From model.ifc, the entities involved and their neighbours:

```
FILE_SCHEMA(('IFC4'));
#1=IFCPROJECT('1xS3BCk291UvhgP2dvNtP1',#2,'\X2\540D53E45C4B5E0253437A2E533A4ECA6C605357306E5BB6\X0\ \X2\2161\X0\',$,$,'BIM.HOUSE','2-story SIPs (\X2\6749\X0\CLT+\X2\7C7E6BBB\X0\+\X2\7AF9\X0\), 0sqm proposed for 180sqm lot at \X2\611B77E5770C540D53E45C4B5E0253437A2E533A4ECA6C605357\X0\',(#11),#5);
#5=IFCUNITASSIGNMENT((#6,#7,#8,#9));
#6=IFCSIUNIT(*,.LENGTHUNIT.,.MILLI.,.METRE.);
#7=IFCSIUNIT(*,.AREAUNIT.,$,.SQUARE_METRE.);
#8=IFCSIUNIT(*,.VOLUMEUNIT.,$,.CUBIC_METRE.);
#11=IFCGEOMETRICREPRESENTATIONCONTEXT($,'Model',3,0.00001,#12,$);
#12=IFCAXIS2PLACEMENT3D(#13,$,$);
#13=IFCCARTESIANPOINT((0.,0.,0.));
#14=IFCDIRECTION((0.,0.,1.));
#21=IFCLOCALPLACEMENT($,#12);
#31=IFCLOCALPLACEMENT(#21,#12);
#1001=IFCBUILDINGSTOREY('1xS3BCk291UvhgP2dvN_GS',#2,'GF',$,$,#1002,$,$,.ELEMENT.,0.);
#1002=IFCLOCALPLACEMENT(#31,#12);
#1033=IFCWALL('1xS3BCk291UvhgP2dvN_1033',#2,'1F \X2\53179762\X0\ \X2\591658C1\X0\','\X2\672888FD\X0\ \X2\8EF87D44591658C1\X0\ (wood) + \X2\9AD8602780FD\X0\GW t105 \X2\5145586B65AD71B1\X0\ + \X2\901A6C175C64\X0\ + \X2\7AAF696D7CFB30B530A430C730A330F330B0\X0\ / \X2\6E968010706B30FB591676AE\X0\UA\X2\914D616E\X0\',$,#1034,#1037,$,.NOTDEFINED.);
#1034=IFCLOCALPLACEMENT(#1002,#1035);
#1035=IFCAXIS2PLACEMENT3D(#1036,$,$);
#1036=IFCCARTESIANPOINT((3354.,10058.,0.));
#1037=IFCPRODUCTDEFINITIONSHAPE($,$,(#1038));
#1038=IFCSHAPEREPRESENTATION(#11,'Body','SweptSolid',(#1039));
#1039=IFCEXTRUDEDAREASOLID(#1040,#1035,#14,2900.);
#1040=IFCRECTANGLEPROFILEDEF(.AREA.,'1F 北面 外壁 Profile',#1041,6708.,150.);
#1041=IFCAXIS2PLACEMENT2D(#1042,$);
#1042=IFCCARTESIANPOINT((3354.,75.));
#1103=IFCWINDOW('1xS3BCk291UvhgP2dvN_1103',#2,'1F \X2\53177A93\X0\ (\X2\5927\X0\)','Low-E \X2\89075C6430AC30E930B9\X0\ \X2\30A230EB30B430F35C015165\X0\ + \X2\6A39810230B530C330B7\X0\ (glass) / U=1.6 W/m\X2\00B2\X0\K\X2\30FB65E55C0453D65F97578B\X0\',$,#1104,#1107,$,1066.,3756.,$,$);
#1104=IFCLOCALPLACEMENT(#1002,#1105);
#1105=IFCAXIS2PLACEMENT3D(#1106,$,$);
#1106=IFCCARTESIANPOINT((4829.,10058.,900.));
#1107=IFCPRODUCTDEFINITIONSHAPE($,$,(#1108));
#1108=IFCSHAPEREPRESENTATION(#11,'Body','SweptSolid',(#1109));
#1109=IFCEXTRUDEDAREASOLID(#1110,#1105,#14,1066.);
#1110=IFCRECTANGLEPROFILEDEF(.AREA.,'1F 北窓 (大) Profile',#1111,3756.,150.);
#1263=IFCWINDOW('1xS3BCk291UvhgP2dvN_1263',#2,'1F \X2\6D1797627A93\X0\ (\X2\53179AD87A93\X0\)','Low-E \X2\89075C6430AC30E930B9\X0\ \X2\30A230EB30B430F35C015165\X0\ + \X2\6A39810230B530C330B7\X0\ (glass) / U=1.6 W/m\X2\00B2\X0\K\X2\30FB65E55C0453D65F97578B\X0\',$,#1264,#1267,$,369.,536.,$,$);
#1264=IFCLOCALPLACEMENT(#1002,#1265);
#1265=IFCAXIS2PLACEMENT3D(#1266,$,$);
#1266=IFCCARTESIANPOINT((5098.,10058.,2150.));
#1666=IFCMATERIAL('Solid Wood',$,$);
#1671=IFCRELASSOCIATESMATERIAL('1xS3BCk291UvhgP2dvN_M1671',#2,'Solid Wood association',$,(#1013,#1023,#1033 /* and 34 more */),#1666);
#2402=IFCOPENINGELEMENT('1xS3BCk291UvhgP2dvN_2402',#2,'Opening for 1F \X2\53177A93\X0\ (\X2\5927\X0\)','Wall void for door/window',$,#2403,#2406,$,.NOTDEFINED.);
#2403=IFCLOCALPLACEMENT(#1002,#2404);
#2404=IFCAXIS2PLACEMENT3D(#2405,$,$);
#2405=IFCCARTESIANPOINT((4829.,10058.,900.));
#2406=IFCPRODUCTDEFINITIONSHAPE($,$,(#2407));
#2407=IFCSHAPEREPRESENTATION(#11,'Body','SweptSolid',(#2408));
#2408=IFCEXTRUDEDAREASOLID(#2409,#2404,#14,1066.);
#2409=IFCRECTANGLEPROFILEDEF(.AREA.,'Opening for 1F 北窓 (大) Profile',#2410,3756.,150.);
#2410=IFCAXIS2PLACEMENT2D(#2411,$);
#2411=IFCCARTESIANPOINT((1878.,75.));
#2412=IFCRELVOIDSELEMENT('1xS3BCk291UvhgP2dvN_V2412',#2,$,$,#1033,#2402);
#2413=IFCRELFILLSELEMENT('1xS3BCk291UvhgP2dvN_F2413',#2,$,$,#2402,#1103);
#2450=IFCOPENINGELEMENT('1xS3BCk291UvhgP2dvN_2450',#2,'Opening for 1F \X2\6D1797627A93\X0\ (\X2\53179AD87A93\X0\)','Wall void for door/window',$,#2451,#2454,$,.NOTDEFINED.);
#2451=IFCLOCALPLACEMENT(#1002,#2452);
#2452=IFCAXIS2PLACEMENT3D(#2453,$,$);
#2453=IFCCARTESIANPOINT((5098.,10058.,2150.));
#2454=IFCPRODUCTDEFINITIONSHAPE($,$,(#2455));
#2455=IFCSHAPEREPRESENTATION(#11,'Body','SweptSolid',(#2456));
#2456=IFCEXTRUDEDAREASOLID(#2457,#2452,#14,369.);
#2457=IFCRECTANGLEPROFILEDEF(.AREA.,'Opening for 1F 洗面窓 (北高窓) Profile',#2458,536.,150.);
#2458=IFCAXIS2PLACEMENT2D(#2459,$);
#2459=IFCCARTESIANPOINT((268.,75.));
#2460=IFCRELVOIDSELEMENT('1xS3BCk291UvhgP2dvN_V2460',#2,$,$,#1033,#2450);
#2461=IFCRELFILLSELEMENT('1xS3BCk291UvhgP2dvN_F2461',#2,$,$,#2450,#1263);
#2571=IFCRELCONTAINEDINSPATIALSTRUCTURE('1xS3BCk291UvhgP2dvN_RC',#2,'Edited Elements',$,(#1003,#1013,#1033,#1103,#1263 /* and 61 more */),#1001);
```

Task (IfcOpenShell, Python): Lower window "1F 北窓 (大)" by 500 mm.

```python
import numpy as np
import ifcopenshell
import ifcopenshell.api.geometry
import ifcopenshell.util.placement
import ifcopenshell.util.unit

model = ifcopenshell.open("model.ifc")
unit_scale = ifcopenshell.util.unit.calculate_unit_scale(model)

window = model.by_guid("1xS3BCk291UvhgP2dvN_1103")
opening = window.FillsVoids[0].RelatingOpeningElement
dz = -0.5 / unit_scale

shift = np.array([0.0, 0.0, dz])
# The window is not placed relative to its opening, so move both.
for product in (opening, window):
    matrix = ifcopenshell.util.placement.get_local_placement(product.ObjectPlacement)
    matrix[:3, 3] += shift
    ifcopenshell.api.geometry.edit_object_placement(model, product=product, matrix=matrix, is_si=False)

print(f"moved by {dz * unit_scale:+.3f} m")

model.write("model_v2.ifc")
```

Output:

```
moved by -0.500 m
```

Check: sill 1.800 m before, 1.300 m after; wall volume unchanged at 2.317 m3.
